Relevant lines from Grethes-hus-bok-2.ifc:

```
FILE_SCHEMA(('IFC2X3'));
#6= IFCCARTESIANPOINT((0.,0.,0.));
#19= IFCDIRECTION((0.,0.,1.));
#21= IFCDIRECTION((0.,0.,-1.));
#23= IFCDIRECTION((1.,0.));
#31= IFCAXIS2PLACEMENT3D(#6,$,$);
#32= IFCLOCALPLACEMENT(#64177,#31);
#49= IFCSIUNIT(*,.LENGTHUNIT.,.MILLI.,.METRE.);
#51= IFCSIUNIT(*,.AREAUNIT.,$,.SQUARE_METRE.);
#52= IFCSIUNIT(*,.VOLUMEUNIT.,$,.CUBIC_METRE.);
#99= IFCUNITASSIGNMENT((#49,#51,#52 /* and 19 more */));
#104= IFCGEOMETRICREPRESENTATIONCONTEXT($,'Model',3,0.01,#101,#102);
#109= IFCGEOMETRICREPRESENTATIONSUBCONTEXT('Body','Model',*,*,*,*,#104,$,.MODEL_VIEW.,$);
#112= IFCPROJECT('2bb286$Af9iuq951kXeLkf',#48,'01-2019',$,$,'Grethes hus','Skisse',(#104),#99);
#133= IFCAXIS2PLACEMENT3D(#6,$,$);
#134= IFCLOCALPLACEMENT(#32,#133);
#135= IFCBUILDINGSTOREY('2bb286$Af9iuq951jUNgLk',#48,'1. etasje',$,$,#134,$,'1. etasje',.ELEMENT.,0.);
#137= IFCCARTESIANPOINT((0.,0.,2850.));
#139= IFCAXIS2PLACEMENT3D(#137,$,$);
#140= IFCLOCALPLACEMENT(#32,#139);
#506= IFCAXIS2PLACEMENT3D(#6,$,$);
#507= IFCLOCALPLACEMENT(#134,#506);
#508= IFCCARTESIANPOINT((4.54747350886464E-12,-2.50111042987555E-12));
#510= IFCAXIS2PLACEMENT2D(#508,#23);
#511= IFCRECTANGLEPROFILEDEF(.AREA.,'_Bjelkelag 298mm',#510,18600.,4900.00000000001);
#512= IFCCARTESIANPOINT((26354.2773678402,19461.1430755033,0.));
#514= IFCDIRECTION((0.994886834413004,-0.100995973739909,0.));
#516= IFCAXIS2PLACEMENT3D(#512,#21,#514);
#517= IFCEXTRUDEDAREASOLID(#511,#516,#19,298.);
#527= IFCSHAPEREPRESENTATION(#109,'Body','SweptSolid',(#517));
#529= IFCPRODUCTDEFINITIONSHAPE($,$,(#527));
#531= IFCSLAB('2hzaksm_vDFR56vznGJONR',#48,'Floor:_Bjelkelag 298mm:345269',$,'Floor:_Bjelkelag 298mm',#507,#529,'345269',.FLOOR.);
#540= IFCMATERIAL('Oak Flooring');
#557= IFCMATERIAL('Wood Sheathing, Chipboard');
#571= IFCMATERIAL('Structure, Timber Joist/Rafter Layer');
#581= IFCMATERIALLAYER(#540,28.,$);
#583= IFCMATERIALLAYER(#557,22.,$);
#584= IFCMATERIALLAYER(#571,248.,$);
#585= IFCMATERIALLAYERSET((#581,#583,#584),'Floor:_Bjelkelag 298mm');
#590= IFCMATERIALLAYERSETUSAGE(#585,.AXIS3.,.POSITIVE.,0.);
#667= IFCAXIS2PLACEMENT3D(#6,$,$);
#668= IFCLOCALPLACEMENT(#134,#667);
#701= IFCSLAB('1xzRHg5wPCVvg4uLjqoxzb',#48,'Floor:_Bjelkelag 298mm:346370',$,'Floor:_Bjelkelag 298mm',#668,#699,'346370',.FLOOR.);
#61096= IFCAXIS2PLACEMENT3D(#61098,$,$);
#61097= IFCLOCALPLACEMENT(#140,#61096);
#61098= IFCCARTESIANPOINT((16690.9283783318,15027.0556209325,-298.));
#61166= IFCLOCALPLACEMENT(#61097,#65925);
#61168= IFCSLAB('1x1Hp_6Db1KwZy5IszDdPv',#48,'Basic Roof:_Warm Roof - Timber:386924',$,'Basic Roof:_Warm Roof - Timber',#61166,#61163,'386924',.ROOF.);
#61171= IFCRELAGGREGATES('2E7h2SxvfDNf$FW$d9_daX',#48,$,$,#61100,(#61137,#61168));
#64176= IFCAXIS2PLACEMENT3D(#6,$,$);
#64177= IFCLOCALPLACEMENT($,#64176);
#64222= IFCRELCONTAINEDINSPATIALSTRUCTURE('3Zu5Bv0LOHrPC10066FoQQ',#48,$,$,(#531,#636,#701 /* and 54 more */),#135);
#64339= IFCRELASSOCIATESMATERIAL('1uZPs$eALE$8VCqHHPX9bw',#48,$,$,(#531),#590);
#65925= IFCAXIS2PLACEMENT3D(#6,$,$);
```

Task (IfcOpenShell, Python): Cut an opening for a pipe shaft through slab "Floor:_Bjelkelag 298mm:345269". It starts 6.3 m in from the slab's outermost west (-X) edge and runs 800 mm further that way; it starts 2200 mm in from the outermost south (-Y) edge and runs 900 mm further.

```python
import numpy as np
import ifcopenshell
import ifcopenshell.api.feature
import ifcopenshell.api.geometry
import ifcopenshell.api.root
import ifcopenshell.geom
import ifcopenshell.util.placement
import ifcopenshell.util.representation
import ifcopenshell.util.shape
import ifcopenshell.util.unit

model = ifcopenshell.open("Grethes-hus-bok-2.ifc")
unit_scale = ifcopenshell.util.unit.calculate_unit_scale(model)
settings = ifcopenshell.geom.settings()


def volume(element):
    """Net volume in cubic metres, openings subtracted."""
    shape = ifcopenshell.geom.create_shape(settings, element)
    return ifcopenshell.util.shape.get_volume(shape.geometry)


slab = model.by_id(531)
before = volume(slab)

# Extent in the slab's own axes, in metres. The edges named are its -X and -Y sides.
slab_shape = ifcopenshell.geom.create_shape(settings, slab)
vertices = ifcopenshell.util.shape.get_vertices(slab_shape.geometry)
x_min, y_min, bottom = vertices.min(axis=0)
top = vertices[:, 2].max()

opening = ifcopenshell.api.root.create_entity(model, ifc_class="IfcOpeningElement", name="Pipe shaft opening")
context = ifcopenshell.util.representation.get_context(model, "Model", "Body", "MODEL_VIEW")
width, depth = 0.8, 0.9
outline = [(0.0, 0.0), (width, 0.0), (width, depth), (0.0, depth), (0.0, 0.0)]
# Overshoot both faces by 50 mm so the cut is clean.
shape = ifcopenshell.api.geometry.add_slab_representation(
    model, context=context, depth=top - bottom + 0.1, polyline=outline
)
ifcopenshell.api.geometry.assign_representation(model, product=opening, representation=shape)

matrix = ifcopenshell.util.placement.get_local_placement(slab.ObjectPlacement)
matrix[:, 3] = matrix @ np.append(np.array([x_min + 6.3, y_min + 2.2, bottom - 0.05]) / unit_scale, 1.0)
ifcopenshell.api.geometry.edit_object_placement(model, product=opening, matrix=matrix, is_si=False)
ifcopenshell.api.feature.add_feature(model, feature=opening, element=slab)

after = volume(slab)

print(f"slab volume {before:.3f} -> {after:.3f} m3")

model.write("Grethes-hus-bok-2-out.ifc")
```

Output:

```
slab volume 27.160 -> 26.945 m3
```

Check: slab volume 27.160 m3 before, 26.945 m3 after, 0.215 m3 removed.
